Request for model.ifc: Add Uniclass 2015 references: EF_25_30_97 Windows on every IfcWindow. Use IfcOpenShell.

First a look at what the model holds.

```python
import ifcopenshell

model = ifcopenshell.open("model.ifc")
print(model.schema)
print("classifications:", [c.Name for c in model.by_type("IfcClassification")])
for ifc_class in ("IfcDoor", "IfcRoof", "IfcStair", "IfcWall", "IfcWindow"):
    print(ifc_class, len(model.by_type(ifc_class)))
```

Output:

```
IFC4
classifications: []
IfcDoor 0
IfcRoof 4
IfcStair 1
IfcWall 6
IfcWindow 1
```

```python
import ifcopenshell
import ifcopenshell.api.classification

model = ifcopenshell.open("model.ifc")

system = ifcopenshell.api.classification.add_classification(model, classification="Uniclass 2015")

codes = {
    "IfcWindow": ("EF_25_30_97", "Windows"),
}
for ifc_class, (code, name) in codes.items():
    products = model.by_type(ifc_class)
    ifcopenshell.api.classification.add_reference(
        model, products=products, classification=system, identification=code, name=name
    )
    print(code, len(products))

model.write("model_v2.ifc")
```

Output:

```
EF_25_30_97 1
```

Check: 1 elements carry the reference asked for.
